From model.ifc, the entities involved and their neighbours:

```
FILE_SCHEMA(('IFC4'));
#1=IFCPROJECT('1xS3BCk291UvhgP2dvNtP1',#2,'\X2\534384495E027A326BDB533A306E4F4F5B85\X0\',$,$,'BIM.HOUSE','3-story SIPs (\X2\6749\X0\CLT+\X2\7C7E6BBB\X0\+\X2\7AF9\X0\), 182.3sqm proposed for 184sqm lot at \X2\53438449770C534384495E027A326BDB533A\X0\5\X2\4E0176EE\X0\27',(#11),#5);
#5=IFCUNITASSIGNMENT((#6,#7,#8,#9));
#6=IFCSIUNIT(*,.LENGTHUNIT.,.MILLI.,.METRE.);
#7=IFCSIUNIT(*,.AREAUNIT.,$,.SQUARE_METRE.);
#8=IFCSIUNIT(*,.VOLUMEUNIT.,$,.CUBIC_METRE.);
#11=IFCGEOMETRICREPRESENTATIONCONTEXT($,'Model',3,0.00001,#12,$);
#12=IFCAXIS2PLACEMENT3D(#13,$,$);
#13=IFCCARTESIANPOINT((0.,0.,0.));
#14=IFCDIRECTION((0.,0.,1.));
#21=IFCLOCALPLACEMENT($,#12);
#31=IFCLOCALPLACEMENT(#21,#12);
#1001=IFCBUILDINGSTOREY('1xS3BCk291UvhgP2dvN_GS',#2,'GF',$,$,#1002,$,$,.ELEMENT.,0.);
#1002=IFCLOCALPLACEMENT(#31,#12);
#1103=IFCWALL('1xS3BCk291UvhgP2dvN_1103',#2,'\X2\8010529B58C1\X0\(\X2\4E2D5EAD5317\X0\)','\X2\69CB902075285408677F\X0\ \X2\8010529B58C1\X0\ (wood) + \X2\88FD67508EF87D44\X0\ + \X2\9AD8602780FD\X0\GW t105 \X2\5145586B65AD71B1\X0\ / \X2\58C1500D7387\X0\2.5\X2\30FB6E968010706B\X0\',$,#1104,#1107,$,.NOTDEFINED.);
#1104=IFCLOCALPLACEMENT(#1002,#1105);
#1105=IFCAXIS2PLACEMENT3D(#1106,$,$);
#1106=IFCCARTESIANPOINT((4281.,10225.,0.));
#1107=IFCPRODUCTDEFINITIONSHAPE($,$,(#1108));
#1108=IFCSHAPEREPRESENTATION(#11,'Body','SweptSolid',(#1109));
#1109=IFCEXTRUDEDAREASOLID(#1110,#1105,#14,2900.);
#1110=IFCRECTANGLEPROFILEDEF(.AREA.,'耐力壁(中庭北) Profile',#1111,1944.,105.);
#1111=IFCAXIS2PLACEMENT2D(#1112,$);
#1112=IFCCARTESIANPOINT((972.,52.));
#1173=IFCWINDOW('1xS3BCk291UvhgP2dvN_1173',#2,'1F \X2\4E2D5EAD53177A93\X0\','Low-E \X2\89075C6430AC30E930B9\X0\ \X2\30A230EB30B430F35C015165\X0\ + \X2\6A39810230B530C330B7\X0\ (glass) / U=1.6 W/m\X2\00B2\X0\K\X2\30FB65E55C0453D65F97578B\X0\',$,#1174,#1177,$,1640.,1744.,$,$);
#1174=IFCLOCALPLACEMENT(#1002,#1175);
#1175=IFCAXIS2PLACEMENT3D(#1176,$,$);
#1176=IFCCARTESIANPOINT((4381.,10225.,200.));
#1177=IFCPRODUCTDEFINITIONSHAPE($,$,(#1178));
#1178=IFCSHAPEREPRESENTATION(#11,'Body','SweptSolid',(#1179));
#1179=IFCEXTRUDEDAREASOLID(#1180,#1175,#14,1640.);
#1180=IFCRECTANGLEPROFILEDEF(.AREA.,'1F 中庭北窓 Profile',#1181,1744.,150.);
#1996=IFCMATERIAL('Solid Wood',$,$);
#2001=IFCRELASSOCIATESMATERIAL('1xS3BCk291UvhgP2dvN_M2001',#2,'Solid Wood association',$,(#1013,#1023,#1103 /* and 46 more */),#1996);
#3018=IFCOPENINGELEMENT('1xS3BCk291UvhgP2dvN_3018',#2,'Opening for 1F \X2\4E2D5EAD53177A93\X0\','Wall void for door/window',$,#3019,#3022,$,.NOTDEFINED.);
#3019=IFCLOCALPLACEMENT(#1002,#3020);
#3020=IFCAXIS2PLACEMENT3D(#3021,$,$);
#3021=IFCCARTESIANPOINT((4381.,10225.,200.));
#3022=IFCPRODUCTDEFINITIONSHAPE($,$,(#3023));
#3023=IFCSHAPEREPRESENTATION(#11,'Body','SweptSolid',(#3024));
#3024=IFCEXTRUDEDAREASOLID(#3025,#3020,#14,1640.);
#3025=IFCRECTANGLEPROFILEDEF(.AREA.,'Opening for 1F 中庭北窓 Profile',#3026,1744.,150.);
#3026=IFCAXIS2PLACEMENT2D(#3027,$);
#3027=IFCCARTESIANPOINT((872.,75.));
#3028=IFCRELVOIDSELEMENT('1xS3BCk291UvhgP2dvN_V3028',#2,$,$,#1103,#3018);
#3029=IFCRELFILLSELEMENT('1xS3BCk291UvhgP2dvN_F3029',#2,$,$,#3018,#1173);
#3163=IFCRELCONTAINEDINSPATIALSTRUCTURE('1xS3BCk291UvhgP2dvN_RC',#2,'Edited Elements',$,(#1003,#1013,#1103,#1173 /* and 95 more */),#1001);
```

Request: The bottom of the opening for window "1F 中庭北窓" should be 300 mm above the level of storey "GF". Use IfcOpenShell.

```python
import numpy as np
import ifcopenshell
import ifcopenshell.api.geometry
import ifcopenshell.geom
import ifcopenshell.util.element
import ifcopenshell.util.placement
import ifcopenshell.util.shape
import ifcopenshell.util.unit

model = ifcopenshell.open("model.ifc")
unit_scale = ifcopenshell.util.unit.calculate_unit_scale(model)

window = model.by_guid("1xS3BCk291UvhgP2dvN_1173")
opening = window.FillsVoids[0].RelatingOpeningElement
storey = ifcopenshell.util.element.get_container(window, ifc_class="IfcBuildingStorey")
level = ifcopenshell.util.placement.get_local_placement(storey.ObjectPlacement)[2, 3]

# The opening's origin need not be at the sill, so measure its lowest point.
shape = ifcopenshell.geom.create_shape(ifcopenshell.geom.settings(), opening)
bottom = ifcopenshell.util.shape.get_shape_bottom_elevation(shape, shape.geometry) / unit_scale
dz = level + 300.0 - bottom

shift = np.array([0.0, 0.0, dz])
# The window is not placed relative to its opening, so move both.
for product in (opening, window):
    matrix = ifcopenshell.util.placement.get_local_placement(product.ObjectPlacement)
    matrix[:3, 3] += shift
    ifcopenshell.api.geometry.edit_object_placement(model, product=product, matrix=matrix, is_si=False)

print(f"moved by {dz * unit_scale:+.3f} m")

model.write("model_edited.ifc")
```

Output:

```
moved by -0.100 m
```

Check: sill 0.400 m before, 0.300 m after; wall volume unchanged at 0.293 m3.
